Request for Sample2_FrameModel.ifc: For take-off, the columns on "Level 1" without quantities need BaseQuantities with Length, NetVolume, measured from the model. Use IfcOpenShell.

First a look at what the model holds.

```python
import ifcopenshell
import ifcopenshell.util.element
import ifcopenshell.util.unit

model = ifcopenshell.open("Sample2_FrameModel.ifc")
print(model.schema)
for unit_type in ("LENGTHUNIT", "AREAUNIT", "VOLUMEUNIT"):
    print(unit_type, ifcopenshell.util.unit.calculate_unit_scale(model, unit_type))
storey = next(s for s in model.by_type("IfcBuildingStorey") if s.Name == "Level 1")
columns = [e for e in ifcopenshell.util.element.get_decomposition(storey) if e.is_a("IfcColumn")]
for e in sorted(columns, key=lambda e: e.id()):
    print(e.id(), e.is_a(), e.Name, list(ifcopenshell.util.element.get_psets(e, qtos_only=True)), sep=" | ")
```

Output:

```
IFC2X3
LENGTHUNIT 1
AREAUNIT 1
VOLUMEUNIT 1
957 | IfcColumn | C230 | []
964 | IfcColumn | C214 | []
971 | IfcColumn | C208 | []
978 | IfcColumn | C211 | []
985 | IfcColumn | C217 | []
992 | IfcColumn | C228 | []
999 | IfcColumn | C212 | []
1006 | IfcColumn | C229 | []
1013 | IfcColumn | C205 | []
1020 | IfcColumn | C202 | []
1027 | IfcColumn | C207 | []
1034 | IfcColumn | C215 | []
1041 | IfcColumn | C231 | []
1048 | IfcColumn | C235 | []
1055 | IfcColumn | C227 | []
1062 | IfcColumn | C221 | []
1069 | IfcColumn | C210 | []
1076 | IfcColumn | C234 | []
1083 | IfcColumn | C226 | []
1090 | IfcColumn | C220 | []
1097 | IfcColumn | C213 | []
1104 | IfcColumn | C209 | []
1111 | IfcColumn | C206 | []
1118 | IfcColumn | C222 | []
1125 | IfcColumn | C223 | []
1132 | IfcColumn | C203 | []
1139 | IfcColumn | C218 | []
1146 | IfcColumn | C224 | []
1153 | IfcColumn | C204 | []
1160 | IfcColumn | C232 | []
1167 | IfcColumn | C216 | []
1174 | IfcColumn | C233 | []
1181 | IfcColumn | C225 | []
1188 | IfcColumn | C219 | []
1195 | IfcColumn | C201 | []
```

```python
import ifcopenshell
import ifcopenshell.api.pset
import ifcopenshell.geom
import ifcopenshell.util.element
import ifcopenshell.util.shape
import ifcopenshell.util.unit

model = ifcopenshell.open("Sample2_FrameModel.ifc")
unit_scale = ifcopenshell.util.unit.calculate_unit_scale(model)
volume_scale = ifcopenshell.util.unit.calculate_unit_scale(model, "VOLUMEUNIT")
settings = ifcopenshell.geom.settings()

storey = next(s for s in model.by_type("IfcBuildingStorey") if s.Name == "Level 1")
columns = [e for e in ifcopenshell.util.element.get_decomposition(storey) if e.is_a("IfcColumn")]

for e in sorted(columns, key=lambda e: e.id()):
    if ifcopenshell.util.element.get_psets(e, qtos_only=True, should_inherit=False):
        continue
    # Geometry comes back in metres, in the element's own axes.
    shape = ifcopenshell.geom.create_shape(settings, e)
    values = {
        "Length": ifcopenshell.util.shape.get_z(shape.geometry) / unit_scale,
        "NetVolume": ifcopenshell.util.shape.get_volume(shape.geometry) / volume_scale,
    }
    qto = ifcopenshell.api.pset.add_qto(model, product=e, name="BaseQuantities")
    ifcopenshell.api.pset.edit_qto(model, qto=qto, properties=values)
    print(e.id(), {k: round(v, 3) for k, v in values.items()})

model.write("Sample2_FrameModel_v2.ifc")
```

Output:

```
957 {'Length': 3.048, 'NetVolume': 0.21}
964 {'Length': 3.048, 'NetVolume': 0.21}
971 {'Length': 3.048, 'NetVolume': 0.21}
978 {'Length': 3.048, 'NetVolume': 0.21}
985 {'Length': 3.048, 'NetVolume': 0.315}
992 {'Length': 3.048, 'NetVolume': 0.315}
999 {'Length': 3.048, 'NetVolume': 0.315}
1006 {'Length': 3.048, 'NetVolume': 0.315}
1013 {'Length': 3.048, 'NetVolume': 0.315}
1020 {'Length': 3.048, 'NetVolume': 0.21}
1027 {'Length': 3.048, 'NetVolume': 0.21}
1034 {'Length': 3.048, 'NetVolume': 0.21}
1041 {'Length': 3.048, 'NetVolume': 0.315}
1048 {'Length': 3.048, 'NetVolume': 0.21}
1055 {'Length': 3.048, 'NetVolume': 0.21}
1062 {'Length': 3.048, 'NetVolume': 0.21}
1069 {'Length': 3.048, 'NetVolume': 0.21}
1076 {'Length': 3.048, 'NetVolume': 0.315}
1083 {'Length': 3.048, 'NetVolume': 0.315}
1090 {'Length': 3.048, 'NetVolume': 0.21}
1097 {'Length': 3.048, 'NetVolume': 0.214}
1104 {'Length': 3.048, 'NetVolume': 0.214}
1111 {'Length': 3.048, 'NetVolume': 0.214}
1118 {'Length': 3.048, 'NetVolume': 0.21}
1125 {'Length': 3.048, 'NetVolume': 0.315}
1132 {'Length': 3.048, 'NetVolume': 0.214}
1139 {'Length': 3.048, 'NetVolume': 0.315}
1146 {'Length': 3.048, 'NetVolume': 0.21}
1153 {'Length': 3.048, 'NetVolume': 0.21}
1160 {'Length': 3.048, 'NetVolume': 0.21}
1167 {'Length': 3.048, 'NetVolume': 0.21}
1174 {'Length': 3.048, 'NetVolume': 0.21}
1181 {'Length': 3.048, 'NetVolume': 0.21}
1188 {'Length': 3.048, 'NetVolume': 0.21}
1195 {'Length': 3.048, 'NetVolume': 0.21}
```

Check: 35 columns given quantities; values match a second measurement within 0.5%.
